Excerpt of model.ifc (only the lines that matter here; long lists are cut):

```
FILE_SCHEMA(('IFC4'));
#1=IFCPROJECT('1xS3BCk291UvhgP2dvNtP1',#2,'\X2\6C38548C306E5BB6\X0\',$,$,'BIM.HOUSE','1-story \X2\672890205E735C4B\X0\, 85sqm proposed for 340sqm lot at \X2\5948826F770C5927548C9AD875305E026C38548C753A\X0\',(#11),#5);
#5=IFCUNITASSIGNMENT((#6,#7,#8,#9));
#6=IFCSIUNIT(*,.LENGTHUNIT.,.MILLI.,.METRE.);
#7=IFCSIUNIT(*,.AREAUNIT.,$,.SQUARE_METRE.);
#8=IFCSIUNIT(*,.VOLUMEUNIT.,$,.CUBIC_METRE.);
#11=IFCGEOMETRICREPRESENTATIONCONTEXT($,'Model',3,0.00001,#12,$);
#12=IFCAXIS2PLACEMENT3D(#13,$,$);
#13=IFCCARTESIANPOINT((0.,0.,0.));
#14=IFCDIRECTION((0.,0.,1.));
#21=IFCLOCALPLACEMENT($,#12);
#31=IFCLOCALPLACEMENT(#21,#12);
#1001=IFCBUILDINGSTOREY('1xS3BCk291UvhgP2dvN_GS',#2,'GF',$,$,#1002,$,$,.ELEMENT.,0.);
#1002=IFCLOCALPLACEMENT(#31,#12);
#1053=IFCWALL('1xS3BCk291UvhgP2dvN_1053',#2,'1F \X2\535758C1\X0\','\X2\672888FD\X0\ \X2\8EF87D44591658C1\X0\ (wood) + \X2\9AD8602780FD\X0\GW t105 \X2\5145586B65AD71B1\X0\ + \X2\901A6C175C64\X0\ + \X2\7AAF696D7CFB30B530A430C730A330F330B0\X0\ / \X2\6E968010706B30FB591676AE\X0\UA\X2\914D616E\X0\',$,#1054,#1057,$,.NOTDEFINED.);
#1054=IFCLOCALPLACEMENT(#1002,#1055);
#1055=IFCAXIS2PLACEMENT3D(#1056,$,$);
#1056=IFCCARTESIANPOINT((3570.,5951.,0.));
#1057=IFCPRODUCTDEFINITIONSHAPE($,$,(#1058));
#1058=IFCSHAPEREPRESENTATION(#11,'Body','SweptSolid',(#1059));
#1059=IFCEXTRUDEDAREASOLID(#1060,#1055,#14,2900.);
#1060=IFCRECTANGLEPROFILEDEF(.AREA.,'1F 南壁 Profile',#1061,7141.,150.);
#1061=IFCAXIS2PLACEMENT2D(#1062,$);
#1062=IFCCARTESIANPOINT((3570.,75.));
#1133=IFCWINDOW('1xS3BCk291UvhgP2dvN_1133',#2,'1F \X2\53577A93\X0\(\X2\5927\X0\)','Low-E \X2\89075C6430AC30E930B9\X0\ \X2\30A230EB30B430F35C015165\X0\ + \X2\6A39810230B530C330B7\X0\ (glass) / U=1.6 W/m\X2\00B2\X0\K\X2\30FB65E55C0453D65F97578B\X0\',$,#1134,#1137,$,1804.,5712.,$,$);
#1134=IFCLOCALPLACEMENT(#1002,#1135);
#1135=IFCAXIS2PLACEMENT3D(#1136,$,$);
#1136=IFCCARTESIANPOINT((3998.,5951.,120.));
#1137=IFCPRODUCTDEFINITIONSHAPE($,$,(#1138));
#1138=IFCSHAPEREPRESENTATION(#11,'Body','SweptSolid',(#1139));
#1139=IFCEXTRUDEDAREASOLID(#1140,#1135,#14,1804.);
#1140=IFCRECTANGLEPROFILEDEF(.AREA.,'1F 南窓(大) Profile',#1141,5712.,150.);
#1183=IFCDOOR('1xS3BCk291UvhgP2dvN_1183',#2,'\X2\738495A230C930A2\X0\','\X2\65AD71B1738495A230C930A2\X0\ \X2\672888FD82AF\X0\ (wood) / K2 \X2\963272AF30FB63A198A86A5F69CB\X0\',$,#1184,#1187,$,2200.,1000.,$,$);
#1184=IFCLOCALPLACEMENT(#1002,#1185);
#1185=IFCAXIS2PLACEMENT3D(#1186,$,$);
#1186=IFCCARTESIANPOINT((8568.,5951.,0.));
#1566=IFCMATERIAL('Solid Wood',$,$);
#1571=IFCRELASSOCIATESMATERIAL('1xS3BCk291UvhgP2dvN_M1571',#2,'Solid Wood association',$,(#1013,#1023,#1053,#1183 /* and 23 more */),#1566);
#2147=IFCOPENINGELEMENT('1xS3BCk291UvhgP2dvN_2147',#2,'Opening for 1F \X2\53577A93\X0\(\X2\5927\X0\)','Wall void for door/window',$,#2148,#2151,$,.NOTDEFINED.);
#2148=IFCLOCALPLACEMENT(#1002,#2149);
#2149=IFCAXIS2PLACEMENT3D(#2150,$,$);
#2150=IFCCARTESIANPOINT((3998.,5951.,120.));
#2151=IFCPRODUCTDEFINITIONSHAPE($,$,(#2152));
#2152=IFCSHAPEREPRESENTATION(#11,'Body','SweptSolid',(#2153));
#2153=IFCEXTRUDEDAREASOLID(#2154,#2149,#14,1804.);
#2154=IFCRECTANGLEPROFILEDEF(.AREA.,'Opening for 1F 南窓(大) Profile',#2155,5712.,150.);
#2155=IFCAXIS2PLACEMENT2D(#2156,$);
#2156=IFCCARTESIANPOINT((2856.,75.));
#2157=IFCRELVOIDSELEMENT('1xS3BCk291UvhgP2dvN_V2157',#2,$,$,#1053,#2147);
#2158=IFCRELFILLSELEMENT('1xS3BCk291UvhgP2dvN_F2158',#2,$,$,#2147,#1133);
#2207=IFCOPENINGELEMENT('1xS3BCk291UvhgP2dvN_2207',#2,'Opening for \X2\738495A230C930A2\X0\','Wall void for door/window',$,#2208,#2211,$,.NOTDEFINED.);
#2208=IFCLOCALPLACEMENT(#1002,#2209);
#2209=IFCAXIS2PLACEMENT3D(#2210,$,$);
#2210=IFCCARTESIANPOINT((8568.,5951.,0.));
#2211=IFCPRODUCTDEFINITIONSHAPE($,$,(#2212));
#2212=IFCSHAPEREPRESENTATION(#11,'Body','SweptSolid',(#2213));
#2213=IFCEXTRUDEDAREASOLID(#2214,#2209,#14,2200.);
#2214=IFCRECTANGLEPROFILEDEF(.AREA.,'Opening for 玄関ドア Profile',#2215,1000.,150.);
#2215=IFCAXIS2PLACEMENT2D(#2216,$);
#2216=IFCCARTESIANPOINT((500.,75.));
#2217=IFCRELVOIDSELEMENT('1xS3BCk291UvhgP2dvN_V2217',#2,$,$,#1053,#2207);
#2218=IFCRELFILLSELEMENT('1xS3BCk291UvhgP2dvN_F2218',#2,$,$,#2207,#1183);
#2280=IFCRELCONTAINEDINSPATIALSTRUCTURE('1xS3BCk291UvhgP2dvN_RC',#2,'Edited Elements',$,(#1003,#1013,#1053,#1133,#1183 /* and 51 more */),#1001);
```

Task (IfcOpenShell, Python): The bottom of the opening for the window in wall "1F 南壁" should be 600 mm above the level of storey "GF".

```python
import numpy as np
import ifcopenshell
import ifcopenshell.api.geometry
import ifcopenshell.geom
import ifcopenshell.util.element
import ifcopenshell.util.placement
import ifcopenshell.util.shape
import ifcopenshell.util.unit

model = ifcopenshell.open("model.ifc")
unit_scale = ifcopenshell.util.unit.calculate_unit_scale(model)

window = model.by_guid("1xS3BCk291UvhgP2dvN_1133")
opening = window.FillsVoids[0].RelatingOpeningElement
storey = ifcopenshell.util.element.get_container(window, ifc_class="IfcBuildingStorey")
level = ifcopenshell.util.placement.get_local_placement(storey.ObjectPlacement)[2, 3]

# The opening's origin need not be at the sill, so measure its lowest point.
shape = ifcopenshell.geom.create_shape(ifcopenshell.geom.settings(), opening)
bottom = ifcopenshell.util.shape.get_shape_bottom_elevation(shape, shape.geometry) / unit_scale
dz = level + 600.0 - bottom

shift = np.array([0.0, 0.0, dz])
# The window is not placed relative to its opening, so move both.
for product in (opening, window):
    matrix = ifcopenshell.util.placement.get_local_placement(product.ObjectPlacement)
    matrix[:3, 3] += shift
    ifcopenshell.api.geometry.edit_object_placement(model, product=product, matrix=matrix, is_si=False)

print(f"moved by {dz * unit_scale:+.3f} m")

model.write("model_updated.ifc")
```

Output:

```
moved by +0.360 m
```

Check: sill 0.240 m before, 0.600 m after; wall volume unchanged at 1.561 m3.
